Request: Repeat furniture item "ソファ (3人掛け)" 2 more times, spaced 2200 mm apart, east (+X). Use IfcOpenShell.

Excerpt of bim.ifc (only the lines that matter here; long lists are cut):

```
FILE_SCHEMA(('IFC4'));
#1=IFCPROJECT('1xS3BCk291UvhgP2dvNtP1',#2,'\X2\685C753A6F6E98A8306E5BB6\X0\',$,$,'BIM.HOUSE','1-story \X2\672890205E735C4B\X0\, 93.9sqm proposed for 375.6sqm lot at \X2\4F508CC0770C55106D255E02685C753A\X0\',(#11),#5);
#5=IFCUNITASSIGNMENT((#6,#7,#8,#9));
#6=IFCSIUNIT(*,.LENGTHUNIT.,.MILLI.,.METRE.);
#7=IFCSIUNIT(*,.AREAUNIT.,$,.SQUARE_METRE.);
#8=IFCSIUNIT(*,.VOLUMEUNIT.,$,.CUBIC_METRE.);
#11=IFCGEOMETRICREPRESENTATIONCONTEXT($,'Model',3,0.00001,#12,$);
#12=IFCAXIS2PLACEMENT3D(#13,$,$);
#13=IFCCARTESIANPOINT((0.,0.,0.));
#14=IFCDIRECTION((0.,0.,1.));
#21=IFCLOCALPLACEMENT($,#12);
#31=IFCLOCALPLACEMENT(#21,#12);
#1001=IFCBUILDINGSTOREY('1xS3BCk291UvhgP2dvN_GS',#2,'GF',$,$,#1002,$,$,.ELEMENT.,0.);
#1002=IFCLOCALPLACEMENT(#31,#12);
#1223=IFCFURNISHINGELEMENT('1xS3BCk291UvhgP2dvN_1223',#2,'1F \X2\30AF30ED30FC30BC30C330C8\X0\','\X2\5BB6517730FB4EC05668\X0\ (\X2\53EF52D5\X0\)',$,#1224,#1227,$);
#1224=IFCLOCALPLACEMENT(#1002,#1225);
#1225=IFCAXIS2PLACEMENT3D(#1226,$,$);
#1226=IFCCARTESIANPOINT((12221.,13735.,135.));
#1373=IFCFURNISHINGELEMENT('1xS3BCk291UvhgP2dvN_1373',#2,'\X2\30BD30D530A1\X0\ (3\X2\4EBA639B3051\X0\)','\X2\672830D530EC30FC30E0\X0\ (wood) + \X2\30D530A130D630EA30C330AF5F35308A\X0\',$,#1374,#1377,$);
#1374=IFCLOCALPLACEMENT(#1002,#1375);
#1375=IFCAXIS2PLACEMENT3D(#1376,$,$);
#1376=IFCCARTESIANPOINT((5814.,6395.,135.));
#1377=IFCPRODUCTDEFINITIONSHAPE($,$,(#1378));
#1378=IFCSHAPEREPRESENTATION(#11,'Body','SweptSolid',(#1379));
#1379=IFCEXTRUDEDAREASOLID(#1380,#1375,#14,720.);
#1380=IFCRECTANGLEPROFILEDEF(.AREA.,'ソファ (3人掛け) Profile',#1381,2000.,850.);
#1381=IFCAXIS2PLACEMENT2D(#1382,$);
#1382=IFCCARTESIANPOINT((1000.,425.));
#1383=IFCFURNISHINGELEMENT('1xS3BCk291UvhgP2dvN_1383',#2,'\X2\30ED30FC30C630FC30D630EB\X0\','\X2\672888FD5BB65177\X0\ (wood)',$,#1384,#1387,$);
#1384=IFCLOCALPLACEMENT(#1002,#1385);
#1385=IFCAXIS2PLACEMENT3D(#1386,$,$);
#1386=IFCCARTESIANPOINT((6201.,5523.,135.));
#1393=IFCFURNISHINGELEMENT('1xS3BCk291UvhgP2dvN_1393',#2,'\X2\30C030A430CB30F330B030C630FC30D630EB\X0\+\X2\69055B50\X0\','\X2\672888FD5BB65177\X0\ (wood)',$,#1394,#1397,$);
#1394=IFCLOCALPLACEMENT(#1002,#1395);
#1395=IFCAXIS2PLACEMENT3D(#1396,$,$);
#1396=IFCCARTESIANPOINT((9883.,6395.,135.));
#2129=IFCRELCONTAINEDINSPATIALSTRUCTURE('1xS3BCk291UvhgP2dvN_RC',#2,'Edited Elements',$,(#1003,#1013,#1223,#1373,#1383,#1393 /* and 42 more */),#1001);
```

```python
import numpy as np
import ifcopenshell
import ifcopenshell.api.geometry
import ifcopenshell.api.root
import ifcopenshell.util.element
import ifcopenshell.util.placement
import ifcopenshell.util.unit

model = ifcopenshell.open("bim.ifc")
unit_scale = ifcopenshell.util.unit.calculate_unit_scale(model)


def reuse_history(source, copy):
    """copy_class also copies each property set's owner history, people and application; keep the originals."""
    for rel in copy.IsDefinedBy:
        if rel.is_a("IfcRelDefinesByProperties") and (history := rel.RelatingPropertyDefinition.OwnerHistory):
            rel.RelatingPropertyDefinition.OwnerHistory = source.OwnerHistory
            ifcopenshell.util.element.remove_deep2(model, history)


source = model.by_guid("1xS3BCk291UvhgP2dvN_1373")
base = ifcopenshell.util.placement.get_local_placement(source.ObjectPlacement)
step = np.array([1.0, 0.0, 0.0]) * 2.2 / unit_scale

for i in range(1, 3):
    copy = ifcopenshell.api.root.copy_class(model, product=source)
    copy.Representation = ifcopenshell.util.element.copy_deep(
        model, source.Representation, exclude=["IfcGeometricRepresentationContext", "IfcRepresentationMap"]
    )
    reuse_history(source, copy)
    matrix = base.copy()
    matrix[:3, 3] += i * step
    print("added at", matrix[:3, 3].round(3) + 0.0)
    ifcopenshell.api.geometry.edit_object_placement(model, product=copy, matrix=matrix, is_si=False)

model.write("bim_rev.ifc")
```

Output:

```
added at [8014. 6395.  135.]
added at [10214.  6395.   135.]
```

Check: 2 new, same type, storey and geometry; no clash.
